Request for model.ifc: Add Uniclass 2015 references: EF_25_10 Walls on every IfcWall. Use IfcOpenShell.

First a look at what the model holds.

```python
import ifcopenshell

model = ifcopenshell.open("model.ifc")
print(model.schema)
print("classifications:", [c.Name for c in model.by_type("IfcClassification")])
for ifc_class in ("IfcDoor", "IfcRoof", "IfcStair", "IfcWall", "IfcWindow"):
    print(ifc_class, len(model.by_type(ifc_class)))
```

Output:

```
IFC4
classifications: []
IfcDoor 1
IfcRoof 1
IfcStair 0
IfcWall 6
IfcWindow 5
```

```python
import ifcopenshell
import ifcopenshell.api.classification

model = ifcopenshell.open("model.ifc")

system = ifcopenshell.api.classification.add_classification(model, classification="Uniclass 2015")

codes = {
    "IfcWall": ("EF_25_10", "Walls"),
}
for ifc_class, (code, name) in codes.items():
    products = model.by_type(ifc_class)
    ifcopenshell.api.classification.add_reference(
        model, products=products, classification=system, identification=code, name=name
    )
    print(code, len(products))

model.write("model-out.ifc")
```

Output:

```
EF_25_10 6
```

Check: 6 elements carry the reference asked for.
